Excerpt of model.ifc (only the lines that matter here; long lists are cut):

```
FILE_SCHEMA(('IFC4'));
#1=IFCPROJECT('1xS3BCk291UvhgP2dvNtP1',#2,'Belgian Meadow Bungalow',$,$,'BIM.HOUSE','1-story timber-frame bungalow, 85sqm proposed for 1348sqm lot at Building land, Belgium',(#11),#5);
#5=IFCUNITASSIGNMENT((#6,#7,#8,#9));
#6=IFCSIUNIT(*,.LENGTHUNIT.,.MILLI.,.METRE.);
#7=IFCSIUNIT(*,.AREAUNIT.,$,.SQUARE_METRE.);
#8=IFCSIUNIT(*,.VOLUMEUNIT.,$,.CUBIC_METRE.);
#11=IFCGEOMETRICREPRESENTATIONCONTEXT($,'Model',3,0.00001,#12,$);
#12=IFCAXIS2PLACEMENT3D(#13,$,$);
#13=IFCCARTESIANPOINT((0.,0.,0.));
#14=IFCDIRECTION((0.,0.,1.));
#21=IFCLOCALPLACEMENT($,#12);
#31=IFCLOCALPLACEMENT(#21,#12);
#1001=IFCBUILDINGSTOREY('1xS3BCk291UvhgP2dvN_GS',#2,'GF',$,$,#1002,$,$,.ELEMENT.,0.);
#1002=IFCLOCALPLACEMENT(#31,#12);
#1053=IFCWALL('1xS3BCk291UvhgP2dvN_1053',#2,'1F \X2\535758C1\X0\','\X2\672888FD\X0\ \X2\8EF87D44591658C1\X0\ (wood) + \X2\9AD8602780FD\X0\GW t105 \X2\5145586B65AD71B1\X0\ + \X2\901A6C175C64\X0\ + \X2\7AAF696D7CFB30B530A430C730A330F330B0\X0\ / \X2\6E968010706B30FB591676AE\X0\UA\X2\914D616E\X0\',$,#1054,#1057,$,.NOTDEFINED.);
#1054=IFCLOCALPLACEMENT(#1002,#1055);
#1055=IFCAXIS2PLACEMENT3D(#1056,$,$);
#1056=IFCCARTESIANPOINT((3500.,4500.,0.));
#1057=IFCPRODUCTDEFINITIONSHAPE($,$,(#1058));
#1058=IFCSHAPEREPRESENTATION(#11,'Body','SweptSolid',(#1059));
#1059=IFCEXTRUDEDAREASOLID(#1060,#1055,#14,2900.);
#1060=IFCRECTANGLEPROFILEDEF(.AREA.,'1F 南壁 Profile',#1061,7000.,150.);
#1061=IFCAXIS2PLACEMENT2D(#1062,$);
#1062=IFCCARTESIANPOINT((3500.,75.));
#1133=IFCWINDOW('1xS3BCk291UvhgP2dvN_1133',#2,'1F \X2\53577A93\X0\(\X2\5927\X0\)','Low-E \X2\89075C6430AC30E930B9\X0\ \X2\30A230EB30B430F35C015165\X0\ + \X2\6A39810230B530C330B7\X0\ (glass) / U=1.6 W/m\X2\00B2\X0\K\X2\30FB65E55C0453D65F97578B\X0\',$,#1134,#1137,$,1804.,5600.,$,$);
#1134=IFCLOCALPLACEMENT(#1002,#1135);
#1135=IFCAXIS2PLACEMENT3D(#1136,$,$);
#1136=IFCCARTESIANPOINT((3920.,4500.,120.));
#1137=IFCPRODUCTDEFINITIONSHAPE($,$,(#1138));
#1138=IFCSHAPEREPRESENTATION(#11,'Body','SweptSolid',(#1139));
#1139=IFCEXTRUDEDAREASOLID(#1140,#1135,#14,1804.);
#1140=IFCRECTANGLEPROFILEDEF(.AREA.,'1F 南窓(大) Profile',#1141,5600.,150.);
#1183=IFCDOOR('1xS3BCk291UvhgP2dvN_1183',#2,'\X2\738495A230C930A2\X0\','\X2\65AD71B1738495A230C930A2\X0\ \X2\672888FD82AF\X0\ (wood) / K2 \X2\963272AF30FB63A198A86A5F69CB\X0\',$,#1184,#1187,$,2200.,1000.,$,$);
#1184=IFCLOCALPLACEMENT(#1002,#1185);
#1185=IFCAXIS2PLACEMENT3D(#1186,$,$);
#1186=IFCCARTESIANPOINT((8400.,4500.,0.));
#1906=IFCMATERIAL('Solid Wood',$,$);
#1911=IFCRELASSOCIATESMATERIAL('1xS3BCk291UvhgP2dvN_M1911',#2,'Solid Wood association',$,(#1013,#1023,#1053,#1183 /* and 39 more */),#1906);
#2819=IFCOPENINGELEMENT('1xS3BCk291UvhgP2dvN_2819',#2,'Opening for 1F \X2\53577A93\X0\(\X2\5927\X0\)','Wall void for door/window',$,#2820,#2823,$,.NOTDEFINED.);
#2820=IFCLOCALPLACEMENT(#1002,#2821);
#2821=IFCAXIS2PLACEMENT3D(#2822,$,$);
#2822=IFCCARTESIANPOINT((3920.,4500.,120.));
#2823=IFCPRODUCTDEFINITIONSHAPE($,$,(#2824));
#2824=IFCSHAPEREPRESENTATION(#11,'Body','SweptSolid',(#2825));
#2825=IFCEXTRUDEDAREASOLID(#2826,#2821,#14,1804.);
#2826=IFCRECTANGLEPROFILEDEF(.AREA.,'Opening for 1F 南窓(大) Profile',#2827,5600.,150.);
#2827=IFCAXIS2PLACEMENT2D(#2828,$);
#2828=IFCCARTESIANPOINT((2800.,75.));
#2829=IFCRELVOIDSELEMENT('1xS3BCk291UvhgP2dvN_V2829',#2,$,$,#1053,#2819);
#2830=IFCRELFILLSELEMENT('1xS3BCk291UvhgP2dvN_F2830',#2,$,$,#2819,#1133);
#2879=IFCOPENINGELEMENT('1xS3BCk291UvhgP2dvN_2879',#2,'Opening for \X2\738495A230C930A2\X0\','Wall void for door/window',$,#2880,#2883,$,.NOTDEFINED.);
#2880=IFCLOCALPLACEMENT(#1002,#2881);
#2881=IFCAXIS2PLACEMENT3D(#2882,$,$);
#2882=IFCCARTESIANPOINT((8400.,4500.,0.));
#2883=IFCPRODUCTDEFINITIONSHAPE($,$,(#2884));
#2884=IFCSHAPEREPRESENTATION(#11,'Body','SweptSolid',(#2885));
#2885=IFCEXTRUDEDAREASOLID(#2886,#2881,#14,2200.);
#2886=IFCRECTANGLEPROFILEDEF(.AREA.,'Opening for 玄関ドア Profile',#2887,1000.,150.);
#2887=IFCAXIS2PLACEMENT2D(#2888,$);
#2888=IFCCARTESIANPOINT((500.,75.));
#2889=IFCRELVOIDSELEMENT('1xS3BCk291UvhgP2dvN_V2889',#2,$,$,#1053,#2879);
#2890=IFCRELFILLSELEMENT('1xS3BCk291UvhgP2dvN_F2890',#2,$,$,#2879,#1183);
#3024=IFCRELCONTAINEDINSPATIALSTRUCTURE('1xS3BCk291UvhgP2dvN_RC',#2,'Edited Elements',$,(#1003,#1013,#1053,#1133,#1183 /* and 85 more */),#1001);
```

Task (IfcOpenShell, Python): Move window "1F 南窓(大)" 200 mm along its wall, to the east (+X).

```python
import ifcopenshell
import ifcopenshell.api.geometry
import ifcopenshell.util.placement
import ifcopenshell.util.unit

model = ifcopenshell.open("model.ifc")
unit_scale = ifcopenshell.util.unit.calculate_unit_scale(model)

window = model.by_guid("1xS3BCk291UvhgP2dvN_1133")
opening = window.FillsVoids[0].RelatingOpeningElement
wall = opening.VoidsElements[0].RelatingBuildingElement

wall_matrix = ifcopenshell.util.placement.get_local_placement(wall.ObjectPlacement)
shift = wall_matrix[:3, 0] * 0.2 / unit_scale
before = ifcopenshell.util.placement.get_local_placement(window.ObjectPlacement)[:3, 3].copy()

# The window is not placed relative to its opening, so move both.
for product in (opening, window):
    matrix = ifcopenshell.util.placement.get_local_placement(product.ObjectPlacement)
    matrix[:3, 3] += shift
    ifcopenshell.api.geometry.edit_object_placement(model, product=product, matrix=matrix, is_si=False)

after = ifcopenshell.util.placement.get_local_placement(window.ObjectPlacement)[:3, 3]
print("window moved by", (after - before).round(3) + 0.0)

model.write("model_updated.ifc")
```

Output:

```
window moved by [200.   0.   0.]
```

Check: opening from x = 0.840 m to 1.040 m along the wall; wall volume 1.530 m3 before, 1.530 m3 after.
